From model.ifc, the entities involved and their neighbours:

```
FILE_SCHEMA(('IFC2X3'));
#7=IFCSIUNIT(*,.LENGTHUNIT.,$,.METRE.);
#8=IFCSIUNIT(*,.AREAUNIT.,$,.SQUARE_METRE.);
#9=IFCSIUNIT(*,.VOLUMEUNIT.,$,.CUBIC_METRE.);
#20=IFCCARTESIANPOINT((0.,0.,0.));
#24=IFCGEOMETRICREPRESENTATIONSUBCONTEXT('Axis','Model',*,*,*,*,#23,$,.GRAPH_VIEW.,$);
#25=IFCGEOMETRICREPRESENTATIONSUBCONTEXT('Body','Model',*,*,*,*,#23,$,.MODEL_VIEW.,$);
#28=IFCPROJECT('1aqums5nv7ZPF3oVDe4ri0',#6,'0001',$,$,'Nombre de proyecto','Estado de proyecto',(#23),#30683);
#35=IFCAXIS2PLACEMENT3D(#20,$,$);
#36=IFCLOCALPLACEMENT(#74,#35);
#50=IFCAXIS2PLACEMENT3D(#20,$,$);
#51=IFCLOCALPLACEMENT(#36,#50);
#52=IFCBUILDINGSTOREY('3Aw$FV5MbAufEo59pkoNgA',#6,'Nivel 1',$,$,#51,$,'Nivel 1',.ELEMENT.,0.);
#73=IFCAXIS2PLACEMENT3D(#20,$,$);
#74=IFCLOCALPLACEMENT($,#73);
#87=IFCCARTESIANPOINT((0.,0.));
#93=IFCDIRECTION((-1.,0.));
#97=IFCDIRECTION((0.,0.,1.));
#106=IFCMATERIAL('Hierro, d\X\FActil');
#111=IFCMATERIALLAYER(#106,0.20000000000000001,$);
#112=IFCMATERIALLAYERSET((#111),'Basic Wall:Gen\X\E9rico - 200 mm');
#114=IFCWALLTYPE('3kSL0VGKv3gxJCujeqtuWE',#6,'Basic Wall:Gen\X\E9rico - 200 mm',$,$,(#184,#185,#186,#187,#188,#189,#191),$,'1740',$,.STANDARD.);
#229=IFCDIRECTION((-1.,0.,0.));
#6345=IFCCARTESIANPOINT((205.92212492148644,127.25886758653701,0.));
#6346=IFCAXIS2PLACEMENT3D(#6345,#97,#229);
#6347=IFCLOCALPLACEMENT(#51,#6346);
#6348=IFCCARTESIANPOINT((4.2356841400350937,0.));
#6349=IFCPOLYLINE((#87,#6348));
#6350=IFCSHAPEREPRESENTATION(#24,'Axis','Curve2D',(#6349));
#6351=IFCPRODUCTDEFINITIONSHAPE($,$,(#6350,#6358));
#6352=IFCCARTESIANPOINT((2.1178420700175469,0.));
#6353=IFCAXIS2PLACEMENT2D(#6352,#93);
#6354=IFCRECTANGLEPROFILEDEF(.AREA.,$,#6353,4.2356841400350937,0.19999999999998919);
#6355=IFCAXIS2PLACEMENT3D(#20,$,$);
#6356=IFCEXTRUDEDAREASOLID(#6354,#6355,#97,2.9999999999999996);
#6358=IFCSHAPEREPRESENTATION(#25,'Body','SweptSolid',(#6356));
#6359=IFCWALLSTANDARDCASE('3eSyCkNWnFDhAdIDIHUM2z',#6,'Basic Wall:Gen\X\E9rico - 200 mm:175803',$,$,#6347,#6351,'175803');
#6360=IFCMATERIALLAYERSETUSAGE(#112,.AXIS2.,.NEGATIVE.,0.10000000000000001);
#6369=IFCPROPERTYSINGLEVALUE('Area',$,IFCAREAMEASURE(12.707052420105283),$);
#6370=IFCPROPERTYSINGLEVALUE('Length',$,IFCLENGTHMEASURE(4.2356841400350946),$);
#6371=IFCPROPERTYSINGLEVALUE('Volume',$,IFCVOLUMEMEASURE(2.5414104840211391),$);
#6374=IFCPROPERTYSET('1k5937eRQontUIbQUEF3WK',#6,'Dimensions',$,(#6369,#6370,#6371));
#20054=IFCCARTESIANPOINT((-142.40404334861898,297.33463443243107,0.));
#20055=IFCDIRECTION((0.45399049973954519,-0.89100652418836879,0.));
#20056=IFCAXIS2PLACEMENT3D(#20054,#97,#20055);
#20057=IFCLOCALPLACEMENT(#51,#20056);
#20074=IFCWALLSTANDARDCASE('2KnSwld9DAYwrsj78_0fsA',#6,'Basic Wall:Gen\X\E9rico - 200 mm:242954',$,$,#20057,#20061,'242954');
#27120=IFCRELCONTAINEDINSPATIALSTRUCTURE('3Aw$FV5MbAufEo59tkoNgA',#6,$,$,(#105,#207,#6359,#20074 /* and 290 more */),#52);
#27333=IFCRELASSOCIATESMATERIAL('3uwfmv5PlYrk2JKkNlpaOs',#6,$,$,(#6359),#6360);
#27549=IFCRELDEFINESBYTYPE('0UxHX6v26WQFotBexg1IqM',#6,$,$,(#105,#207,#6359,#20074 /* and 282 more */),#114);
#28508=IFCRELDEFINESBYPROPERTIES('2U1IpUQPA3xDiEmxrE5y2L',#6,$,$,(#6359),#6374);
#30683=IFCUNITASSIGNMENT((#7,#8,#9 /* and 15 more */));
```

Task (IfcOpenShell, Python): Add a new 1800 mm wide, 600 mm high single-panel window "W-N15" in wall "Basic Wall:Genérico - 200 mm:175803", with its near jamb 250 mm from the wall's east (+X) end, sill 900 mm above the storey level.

```python
import numpy as np
import ifcopenshell
import ifcopenshell.api.feature
import ifcopenshell.api.geometry
import ifcopenshell.api.pset
import ifcopenshell.api.root
import ifcopenshell.api.spatial
import ifcopenshell.api.type
import ifcopenshell.geom
import ifcopenshell.util.element
import ifcopenshell.util.placement
import ifcopenshell.util.representation
import ifcopenshell.util.shape
import ifcopenshell.util.unit

model = ifcopenshell.open("model.ifc")
unit_scale = ifcopenshell.util.unit.calculate_unit_scale(model)
area_scale = ifcopenshell.util.unit.calculate_unit_scale(model, "AREAUNIT")
volume_scale = ifcopenshell.util.unit.calculate_unit_scale(model, "VOLUMEUNIT")
settings = ifcopenshell.geom.settings()


def volume(element):
    """Net volume in cubic metres, openings subtracted."""
    shape = ifcopenshell.geom.create_shape(settings, element)
    return ifcopenshell.util.shape.get_volume(shape.geometry)


wall = model.by_guid("3eSyCkNWnFDhAdIDIHUM2z")
storey = ifcopenshell.util.element.get_container(wall, ifc_class="IfcBuildingStorey")
context = ifcopenshell.util.representation.get_context(model, "Model", "Body", "MODEL_VIEW")
before = volume(wall)

width, height, from_end, sill = 1.8, 0.6, 0.25, 0.9  # metres

# The wall runs along its own X axis, and the end named is its -X end.
wall_shape = ifcopenshell.geom.create_shape(settings, wall)
x, y, z = ifcopenshell.util.shape.get_vertices(wall_shape.geometry).T
start = x.min() + from_end
face, thickness = float(y.min()), float(y.max() - y.min())
wall_matrix = ifcopenshell.util.placement.get_local_placement(wall.ObjectPlacement)
level = ifcopenshell.util.placement.get_local_placement(storey.ObjectPlacement)[2, 3]


def in_wall(x, y):
    """Placement at x, y metres in the wall's axes, at sill height."""
    matrix = wall_matrix.copy()
    matrix[:, 3] = wall_matrix @ np.array([x / unit_scale, y / unit_scale, 0.0, 1.0])
    matrix[2, 3] = level + sill / unit_scale
    return matrix


# Opening: a box that overshoots both wall faces by 50 mm.
opening = ifcopenshell.api.root.create_entity(model, ifc_class="IfcOpeningElement")
box = ifcopenshell.api.geometry.add_wall_representation(
    model, context=context, length=width, height=height, thickness=thickness + 0.1
)
ifcopenshell.api.geometry.assign_representation(model, product=opening, representation=box)
ifcopenshell.api.geometry.edit_object_placement(model, product=opening, matrix=in_wall(start, face - 0.05), is_si=False)
ifcopenshell.api.feature.add_feature(model, feature=opening, element=wall)

window = ifcopenshell.api.root.create_entity(model, ifc_class="IfcWindow", name="W-N15")
window.OverallWidth, window.OverallHeight = width / unit_scale, height / unit_scale
body = ifcopenshell.api.geometry.add_window_representation(
    model,
    context=context,
    overall_width=window.OverallWidth,
    overall_height=window.OverallHeight,
    partition_type="SINGLE_PANEL",
)
ifcopenshell.api.geometry.assign_representation(model, product=window, representation=body)
ifcopenshell.api.spatial.assign_container(model, products=[window], relating_structure=storey)
fills = ifcopenshell.api.feature.add_filling(model, opening=opening, element=window)
fills.OwnerHistory = window.OwnerHistory  # required in IFC2X3

# IFC2X3 keeps the operation on the window style.
style = ifcopenshell.api.root.create_entity(model, ifc_class="IfcWindowStyle", name="W-N15")
style.OperationType, style.ConstructionType = "SINGLE_PANEL", "NOTDEFINED"
style.ParameterTakesPrecedence = style.Sizeable = False
ifcopenshell.api.type.assign_type(model, related_objects=[window], relating_type=style)

# Centre the window in the wall's thickness.
ifcopenshell.api.geometry.edit_object_placement(model, product=window, matrix=in_wall(start, face), is_si=False)
window_shape = ifcopenshell.geom.create_shape(settings, window)
depth = ifcopenshell.util.shape.get_vertices(window_shape.geometry)[:, 1]
offset = face + thickness / 2 - (depth.min() + depth.max()) / 2
ifcopenshell.api.geometry.edit_object_placement(model, product=window, matrix=in_wall(start, offset), is_si=False)

after = volume(wall)

# Update the wall's stored quantities.
pset = model.by_id(ifcopenshell.util.element.get_pset(wall, "Dimensions", should_inherit=False)["id"])
ifcopenshell.api.pset.edit_pset(model, pset=pset, properties={
    "Area": model.create_entity("IfcAreaMeasure", after / thickness / area_scale),
    "Volume": model.create_entity("IfcVolumeMeasure", after / volume_scale),
})

print(f"wall volume {before:.3f} -> {after:.3f} m3")

model.write("model_edited.ifc")
```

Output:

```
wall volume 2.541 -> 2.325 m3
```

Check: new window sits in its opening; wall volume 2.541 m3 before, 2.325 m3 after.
